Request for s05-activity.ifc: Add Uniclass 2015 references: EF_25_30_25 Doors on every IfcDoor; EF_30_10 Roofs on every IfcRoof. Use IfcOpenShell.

First a look at what the model holds.

```python
import ifcopenshell

model = ifcopenshell.open("s05-activity.ifc")
print(model.schema)
print("classifications:", [c.Name for c in model.by_type("IfcClassification")])
for ifc_class in ("IfcDoor", "IfcRoof", "IfcStair", "IfcWall", "IfcWindow"):
    print(ifc_class, len(model.by_type(ifc_class)))
```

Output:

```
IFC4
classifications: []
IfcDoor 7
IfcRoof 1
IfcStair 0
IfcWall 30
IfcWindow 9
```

```python
import ifcopenshell
import ifcopenshell.api.classification

model = ifcopenshell.open("s05-activity.ifc")

system = ifcopenshell.api.classification.add_classification(model, classification="Uniclass 2015")

codes = {
    "IfcDoor": ("EF_25_30_25", "Doors"),
    "IfcRoof": ("EF_30_10", "Roofs"),
}
for ifc_class, (code, name) in codes.items():
    products = model.by_type(ifc_class)
    ifcopenshell.api.classification.add_reference(
        model, products=products, classification=system, identification=code, name=name
    )
    print(code, len(products))

model.write("s05-activity_edited.ifc")
```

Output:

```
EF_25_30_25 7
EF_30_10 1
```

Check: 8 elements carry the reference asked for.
